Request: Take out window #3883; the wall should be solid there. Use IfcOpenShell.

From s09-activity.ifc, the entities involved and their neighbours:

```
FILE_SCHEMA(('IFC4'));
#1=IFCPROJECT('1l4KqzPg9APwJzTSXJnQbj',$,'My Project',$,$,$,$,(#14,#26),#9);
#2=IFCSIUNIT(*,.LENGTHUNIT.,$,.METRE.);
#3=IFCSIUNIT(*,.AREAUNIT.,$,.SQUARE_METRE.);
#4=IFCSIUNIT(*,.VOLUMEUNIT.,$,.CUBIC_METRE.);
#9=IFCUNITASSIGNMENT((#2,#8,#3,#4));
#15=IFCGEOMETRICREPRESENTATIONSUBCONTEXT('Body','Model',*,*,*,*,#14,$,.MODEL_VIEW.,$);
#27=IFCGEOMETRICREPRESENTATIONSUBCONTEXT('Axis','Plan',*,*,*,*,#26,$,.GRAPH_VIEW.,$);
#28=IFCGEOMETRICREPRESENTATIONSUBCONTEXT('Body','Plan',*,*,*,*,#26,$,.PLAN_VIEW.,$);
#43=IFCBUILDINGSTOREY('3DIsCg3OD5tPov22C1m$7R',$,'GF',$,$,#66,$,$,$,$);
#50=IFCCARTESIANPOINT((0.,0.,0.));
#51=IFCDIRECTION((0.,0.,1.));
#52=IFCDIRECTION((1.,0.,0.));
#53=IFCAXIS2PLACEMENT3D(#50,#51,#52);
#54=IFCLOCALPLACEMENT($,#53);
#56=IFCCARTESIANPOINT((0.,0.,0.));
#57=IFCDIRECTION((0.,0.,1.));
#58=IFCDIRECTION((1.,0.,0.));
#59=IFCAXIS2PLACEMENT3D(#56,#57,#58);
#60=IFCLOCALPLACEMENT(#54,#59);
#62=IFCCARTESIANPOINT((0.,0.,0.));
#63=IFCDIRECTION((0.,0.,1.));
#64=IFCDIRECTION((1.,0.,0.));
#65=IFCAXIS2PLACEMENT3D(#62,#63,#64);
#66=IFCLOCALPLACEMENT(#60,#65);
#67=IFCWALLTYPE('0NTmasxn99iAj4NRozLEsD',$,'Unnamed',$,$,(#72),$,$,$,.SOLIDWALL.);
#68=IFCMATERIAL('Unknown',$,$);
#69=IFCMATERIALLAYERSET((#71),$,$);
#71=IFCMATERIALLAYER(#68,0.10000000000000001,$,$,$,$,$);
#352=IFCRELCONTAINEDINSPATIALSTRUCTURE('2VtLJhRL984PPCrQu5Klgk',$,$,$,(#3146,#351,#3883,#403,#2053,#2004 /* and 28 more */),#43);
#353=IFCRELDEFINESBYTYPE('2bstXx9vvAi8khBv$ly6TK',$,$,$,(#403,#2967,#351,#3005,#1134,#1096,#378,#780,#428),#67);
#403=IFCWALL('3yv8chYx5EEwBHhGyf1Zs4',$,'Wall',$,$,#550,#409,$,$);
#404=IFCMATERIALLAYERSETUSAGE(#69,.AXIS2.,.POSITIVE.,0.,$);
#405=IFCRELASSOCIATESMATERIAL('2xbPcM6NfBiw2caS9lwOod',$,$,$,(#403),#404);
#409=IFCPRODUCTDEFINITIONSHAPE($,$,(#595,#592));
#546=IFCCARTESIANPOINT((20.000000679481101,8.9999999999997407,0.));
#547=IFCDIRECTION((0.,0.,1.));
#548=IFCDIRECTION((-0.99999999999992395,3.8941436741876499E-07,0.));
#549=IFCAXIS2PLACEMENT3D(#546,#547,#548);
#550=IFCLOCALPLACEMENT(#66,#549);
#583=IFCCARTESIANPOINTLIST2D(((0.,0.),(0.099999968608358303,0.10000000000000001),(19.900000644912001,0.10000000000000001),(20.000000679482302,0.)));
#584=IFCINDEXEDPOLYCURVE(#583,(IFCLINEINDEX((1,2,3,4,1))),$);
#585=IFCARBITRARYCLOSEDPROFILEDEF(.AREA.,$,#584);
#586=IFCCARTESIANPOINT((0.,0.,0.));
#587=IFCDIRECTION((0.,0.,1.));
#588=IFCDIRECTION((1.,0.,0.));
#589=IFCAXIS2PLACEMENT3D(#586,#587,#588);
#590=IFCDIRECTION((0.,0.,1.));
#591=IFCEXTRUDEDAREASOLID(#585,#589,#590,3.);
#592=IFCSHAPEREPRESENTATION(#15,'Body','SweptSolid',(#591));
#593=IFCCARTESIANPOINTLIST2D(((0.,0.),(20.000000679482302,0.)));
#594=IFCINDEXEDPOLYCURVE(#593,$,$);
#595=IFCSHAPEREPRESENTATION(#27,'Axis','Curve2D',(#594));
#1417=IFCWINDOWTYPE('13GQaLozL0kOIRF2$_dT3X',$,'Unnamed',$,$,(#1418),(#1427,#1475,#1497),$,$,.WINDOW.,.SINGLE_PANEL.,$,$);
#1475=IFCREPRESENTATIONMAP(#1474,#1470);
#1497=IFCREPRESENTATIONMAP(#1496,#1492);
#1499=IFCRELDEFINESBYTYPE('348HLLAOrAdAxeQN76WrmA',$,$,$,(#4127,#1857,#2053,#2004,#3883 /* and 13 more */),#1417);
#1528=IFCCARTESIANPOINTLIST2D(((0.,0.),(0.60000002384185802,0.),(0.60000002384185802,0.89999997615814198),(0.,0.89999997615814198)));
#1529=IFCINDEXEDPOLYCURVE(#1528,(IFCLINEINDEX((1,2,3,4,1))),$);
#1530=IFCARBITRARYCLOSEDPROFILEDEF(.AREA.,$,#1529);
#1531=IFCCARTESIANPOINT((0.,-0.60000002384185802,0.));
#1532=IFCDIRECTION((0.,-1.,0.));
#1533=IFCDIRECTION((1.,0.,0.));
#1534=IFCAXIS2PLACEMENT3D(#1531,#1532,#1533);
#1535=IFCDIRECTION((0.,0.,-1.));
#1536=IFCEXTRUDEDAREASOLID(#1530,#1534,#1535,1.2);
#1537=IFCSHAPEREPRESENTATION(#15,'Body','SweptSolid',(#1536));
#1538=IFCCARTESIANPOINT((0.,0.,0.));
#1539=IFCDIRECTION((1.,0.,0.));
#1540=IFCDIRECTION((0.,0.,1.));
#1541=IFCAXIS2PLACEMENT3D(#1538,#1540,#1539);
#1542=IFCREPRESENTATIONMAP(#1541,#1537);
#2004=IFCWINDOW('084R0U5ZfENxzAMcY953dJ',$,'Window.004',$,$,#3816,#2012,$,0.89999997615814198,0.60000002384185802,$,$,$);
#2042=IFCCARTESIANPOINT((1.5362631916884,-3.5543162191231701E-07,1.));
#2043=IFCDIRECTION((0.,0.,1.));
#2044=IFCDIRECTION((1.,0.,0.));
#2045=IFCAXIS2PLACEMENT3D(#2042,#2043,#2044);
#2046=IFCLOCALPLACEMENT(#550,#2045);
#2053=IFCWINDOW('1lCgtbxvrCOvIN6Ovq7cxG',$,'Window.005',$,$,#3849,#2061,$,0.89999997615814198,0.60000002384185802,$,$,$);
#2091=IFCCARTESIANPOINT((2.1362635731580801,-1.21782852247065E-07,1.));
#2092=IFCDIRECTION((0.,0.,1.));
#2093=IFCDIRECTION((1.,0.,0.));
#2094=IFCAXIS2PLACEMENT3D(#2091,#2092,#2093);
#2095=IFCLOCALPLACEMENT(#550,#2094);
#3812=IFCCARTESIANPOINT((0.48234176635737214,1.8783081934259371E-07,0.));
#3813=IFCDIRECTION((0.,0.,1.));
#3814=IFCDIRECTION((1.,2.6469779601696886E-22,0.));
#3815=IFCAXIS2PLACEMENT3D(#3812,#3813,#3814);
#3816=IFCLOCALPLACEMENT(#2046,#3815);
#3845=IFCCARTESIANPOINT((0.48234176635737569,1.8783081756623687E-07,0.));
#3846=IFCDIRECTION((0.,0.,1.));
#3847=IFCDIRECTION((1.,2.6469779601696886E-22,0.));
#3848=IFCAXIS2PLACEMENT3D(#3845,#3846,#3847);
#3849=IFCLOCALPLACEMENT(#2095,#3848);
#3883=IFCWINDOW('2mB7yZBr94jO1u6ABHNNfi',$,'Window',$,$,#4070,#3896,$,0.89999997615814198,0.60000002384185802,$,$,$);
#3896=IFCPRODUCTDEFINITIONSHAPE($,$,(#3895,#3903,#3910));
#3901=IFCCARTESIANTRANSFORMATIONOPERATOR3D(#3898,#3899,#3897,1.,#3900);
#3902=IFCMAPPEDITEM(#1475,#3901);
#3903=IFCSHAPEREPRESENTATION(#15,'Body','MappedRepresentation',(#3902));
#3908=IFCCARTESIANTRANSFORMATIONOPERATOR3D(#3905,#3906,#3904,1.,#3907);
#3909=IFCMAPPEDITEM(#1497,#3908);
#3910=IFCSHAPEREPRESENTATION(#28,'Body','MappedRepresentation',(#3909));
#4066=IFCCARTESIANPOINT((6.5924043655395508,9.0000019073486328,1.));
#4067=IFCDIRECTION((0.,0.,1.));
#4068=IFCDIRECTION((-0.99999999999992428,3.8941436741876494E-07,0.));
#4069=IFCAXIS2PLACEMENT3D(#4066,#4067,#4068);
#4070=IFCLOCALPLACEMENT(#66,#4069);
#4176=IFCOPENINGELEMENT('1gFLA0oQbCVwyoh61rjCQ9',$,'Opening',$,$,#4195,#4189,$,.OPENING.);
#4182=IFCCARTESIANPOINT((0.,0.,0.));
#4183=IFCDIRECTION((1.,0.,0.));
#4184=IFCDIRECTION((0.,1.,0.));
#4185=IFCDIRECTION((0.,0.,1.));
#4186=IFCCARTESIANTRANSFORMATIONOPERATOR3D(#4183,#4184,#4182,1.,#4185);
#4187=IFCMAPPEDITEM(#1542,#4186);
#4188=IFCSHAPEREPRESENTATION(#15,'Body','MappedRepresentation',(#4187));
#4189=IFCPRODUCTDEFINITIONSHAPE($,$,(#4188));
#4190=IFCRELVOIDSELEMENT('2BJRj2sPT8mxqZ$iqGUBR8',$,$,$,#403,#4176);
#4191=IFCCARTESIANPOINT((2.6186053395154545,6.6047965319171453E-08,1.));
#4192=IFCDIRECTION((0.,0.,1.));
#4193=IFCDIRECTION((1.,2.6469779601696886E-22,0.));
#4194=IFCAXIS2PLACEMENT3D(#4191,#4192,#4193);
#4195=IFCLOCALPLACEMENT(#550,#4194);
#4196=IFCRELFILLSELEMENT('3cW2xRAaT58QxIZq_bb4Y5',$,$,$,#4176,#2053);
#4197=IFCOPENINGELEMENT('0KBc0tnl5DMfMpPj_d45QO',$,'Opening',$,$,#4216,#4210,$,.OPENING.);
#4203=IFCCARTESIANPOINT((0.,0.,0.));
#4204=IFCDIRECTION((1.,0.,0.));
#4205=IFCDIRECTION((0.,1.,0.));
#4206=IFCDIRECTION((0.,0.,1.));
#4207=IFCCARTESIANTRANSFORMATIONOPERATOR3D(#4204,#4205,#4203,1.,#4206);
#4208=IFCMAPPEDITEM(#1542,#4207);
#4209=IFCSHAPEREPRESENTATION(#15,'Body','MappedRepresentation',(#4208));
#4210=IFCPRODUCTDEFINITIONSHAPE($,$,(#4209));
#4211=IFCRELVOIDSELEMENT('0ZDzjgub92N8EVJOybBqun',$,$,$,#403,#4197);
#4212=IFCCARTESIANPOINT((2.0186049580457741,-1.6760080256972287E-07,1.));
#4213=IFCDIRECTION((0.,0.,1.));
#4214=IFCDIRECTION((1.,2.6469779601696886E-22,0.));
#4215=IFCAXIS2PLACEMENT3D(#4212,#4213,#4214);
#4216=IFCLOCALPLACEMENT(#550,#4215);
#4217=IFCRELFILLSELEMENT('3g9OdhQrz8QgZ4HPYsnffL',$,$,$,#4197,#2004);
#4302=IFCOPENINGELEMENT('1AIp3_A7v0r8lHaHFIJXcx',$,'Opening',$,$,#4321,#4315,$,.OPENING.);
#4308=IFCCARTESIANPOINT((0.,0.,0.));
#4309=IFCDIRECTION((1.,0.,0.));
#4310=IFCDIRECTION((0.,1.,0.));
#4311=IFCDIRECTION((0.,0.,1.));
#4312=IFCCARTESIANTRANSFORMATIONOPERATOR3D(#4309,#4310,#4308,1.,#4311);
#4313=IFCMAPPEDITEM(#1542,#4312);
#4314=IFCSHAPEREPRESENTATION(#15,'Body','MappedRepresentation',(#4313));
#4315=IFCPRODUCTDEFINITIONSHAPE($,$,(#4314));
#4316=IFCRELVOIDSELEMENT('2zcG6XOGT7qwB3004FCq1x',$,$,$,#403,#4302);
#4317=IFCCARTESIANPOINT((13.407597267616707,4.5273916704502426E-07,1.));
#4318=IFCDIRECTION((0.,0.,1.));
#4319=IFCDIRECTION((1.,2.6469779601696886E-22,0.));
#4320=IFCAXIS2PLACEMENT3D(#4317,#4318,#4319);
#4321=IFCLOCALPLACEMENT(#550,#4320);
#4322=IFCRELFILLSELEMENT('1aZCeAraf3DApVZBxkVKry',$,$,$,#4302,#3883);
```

```python
import ifcopenshell
import ifcopenshell.api.feature
import ifcopenshell.api.root
import ifcopenshell.geom
import ifcopenshell.util.shape

model = ifcopenshell.open("s09-activity.ifc")
settings = ifcopenshell.geom.settings()


def volume(element):
    """Net volume in cubic metres, openings subtracted."""
    shape = ifcopenshell.geom.create_shape(settings, element)
    return ifcopenshell.util.shape.get_volume(shape.geometry)


window = model.by_guid("2mB7yZBr94jO1u6ABHNNfi")
opening = window.FillsVoids[0].RelatingOpeningElement
wall = opening.VoidsElements[0].RelatingBuildingElement
before = volume(wall)

ifcopenshell.api.root.remove_product(model, product=window)
ifcopenshell.api.feature.remove_feature(model, feature=opening)

after = volume(wall)

print(f"wall volume {before:.3f} -> {after:.3f} m3")

model.write("s09-activity_updated.ifc")
```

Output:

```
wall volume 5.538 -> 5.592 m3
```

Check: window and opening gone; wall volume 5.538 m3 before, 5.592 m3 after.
